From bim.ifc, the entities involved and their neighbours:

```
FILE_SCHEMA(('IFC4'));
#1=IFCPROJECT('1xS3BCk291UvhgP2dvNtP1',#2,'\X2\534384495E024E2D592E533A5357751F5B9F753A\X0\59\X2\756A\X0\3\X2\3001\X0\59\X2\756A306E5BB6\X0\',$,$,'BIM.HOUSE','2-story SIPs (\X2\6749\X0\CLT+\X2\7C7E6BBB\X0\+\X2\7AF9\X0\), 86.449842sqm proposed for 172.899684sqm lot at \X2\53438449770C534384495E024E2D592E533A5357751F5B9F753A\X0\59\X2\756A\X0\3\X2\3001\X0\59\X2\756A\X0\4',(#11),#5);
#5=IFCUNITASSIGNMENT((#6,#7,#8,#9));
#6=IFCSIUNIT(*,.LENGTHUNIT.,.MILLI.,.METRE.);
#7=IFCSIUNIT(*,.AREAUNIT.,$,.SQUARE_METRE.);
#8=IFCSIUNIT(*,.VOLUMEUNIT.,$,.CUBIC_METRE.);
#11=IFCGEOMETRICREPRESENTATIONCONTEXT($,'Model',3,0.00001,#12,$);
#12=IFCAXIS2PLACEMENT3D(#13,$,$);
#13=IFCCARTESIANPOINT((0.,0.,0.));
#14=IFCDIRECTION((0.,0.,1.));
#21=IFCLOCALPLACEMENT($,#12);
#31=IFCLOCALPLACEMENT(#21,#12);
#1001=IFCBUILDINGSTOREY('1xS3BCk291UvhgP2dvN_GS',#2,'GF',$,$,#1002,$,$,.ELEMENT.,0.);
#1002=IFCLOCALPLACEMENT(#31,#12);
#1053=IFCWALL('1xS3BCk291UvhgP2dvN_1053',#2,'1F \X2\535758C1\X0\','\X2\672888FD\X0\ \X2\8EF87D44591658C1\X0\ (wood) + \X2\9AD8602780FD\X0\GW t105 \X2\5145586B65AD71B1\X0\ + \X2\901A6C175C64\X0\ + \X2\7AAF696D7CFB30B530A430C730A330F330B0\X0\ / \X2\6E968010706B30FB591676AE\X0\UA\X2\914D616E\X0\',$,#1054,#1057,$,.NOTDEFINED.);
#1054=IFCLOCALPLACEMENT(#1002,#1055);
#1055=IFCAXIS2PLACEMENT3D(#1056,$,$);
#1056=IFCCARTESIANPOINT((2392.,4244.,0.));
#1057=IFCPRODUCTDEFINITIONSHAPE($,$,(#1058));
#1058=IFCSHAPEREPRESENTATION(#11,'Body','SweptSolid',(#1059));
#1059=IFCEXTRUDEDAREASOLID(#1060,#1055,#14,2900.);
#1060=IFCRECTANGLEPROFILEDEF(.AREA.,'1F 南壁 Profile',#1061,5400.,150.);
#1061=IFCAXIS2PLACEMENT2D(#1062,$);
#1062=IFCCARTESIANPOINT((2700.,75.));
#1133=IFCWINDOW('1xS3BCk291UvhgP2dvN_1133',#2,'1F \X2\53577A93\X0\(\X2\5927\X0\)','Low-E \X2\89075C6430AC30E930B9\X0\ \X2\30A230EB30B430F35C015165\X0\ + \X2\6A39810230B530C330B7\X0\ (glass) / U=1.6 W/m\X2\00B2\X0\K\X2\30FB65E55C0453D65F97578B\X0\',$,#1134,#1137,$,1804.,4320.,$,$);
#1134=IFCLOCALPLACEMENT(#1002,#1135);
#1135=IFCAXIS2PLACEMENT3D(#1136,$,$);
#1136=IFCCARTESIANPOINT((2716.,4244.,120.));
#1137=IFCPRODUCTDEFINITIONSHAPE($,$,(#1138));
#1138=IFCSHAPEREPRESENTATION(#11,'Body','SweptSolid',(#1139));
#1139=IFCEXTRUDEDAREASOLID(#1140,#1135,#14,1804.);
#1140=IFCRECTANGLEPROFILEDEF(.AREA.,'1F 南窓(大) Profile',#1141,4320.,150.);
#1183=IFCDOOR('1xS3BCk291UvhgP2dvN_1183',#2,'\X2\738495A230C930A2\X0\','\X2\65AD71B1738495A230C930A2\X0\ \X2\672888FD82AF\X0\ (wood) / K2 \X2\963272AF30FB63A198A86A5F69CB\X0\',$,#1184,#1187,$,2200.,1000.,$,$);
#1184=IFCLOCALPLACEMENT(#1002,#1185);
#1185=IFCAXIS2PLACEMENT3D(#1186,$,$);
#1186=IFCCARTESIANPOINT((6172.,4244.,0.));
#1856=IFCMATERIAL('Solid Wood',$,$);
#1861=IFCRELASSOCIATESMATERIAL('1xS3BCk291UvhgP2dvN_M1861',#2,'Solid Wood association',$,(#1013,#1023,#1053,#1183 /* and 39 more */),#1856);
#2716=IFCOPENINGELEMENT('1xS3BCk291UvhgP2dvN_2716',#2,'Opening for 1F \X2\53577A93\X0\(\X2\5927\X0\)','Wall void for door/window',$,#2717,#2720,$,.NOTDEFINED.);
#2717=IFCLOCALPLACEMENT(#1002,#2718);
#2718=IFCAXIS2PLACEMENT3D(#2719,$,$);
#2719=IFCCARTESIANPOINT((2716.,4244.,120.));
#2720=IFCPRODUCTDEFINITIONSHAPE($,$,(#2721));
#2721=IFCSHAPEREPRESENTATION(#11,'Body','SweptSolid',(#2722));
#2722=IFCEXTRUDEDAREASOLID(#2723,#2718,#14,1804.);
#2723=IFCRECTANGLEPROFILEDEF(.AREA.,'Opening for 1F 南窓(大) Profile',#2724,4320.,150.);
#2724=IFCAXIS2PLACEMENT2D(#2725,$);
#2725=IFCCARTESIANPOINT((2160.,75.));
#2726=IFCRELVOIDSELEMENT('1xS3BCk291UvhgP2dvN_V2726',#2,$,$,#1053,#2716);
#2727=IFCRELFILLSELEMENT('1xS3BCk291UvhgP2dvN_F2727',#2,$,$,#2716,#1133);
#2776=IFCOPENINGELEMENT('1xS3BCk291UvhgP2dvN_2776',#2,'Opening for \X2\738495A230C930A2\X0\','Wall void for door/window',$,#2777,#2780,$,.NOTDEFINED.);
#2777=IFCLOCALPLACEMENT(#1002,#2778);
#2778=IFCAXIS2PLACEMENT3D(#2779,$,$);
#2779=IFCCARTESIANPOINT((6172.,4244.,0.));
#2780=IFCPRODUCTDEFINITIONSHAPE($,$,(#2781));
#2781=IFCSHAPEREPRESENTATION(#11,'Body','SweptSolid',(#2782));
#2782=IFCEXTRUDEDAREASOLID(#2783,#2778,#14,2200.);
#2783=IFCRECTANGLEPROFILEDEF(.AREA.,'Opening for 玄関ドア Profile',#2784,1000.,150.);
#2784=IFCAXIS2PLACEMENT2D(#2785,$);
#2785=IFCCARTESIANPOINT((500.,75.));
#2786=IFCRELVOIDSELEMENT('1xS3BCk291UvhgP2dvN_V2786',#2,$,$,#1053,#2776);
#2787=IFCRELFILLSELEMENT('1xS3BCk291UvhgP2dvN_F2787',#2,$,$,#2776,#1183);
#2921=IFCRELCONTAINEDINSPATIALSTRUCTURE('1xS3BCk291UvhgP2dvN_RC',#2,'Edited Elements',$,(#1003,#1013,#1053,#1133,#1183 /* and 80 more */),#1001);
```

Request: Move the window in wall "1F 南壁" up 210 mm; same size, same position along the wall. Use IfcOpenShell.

```python
import numpy as np
import ifcopenshell
import ifcopenshell.api.geometry
import ifcopenshell.util.placement
import ifcopenshell.util.unit

model = ifcopenshell.open("bim.ifc")
unit_scale = ifcopenshell.util.unit.calculate_unit_scale(model)

window = model.by_guid("1xS3BCk291UvhgP2dvN_1133")
opening = window.FillsVoids[0].RelatingOpeningElement
dz = 210.0

shift = np.array([0.0, 0.0, dz])
# The window is not placed relative to its opening, so move both.
for product in (opening, window):
    matrix = ifcopenshell.util.placement.get_local_placement(product.ObjectPlacement)
    matrix[:3, 3] += shift
    ifcopenshell.api.geometry.edit_object_placement(model, product=product, matrix=matrix, is_si=False)

print(f"moved by {dz * unit_scale:+.3f} m")

model.write("bim_v2.ifc")
```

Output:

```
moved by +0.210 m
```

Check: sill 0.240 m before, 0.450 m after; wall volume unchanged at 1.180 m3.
